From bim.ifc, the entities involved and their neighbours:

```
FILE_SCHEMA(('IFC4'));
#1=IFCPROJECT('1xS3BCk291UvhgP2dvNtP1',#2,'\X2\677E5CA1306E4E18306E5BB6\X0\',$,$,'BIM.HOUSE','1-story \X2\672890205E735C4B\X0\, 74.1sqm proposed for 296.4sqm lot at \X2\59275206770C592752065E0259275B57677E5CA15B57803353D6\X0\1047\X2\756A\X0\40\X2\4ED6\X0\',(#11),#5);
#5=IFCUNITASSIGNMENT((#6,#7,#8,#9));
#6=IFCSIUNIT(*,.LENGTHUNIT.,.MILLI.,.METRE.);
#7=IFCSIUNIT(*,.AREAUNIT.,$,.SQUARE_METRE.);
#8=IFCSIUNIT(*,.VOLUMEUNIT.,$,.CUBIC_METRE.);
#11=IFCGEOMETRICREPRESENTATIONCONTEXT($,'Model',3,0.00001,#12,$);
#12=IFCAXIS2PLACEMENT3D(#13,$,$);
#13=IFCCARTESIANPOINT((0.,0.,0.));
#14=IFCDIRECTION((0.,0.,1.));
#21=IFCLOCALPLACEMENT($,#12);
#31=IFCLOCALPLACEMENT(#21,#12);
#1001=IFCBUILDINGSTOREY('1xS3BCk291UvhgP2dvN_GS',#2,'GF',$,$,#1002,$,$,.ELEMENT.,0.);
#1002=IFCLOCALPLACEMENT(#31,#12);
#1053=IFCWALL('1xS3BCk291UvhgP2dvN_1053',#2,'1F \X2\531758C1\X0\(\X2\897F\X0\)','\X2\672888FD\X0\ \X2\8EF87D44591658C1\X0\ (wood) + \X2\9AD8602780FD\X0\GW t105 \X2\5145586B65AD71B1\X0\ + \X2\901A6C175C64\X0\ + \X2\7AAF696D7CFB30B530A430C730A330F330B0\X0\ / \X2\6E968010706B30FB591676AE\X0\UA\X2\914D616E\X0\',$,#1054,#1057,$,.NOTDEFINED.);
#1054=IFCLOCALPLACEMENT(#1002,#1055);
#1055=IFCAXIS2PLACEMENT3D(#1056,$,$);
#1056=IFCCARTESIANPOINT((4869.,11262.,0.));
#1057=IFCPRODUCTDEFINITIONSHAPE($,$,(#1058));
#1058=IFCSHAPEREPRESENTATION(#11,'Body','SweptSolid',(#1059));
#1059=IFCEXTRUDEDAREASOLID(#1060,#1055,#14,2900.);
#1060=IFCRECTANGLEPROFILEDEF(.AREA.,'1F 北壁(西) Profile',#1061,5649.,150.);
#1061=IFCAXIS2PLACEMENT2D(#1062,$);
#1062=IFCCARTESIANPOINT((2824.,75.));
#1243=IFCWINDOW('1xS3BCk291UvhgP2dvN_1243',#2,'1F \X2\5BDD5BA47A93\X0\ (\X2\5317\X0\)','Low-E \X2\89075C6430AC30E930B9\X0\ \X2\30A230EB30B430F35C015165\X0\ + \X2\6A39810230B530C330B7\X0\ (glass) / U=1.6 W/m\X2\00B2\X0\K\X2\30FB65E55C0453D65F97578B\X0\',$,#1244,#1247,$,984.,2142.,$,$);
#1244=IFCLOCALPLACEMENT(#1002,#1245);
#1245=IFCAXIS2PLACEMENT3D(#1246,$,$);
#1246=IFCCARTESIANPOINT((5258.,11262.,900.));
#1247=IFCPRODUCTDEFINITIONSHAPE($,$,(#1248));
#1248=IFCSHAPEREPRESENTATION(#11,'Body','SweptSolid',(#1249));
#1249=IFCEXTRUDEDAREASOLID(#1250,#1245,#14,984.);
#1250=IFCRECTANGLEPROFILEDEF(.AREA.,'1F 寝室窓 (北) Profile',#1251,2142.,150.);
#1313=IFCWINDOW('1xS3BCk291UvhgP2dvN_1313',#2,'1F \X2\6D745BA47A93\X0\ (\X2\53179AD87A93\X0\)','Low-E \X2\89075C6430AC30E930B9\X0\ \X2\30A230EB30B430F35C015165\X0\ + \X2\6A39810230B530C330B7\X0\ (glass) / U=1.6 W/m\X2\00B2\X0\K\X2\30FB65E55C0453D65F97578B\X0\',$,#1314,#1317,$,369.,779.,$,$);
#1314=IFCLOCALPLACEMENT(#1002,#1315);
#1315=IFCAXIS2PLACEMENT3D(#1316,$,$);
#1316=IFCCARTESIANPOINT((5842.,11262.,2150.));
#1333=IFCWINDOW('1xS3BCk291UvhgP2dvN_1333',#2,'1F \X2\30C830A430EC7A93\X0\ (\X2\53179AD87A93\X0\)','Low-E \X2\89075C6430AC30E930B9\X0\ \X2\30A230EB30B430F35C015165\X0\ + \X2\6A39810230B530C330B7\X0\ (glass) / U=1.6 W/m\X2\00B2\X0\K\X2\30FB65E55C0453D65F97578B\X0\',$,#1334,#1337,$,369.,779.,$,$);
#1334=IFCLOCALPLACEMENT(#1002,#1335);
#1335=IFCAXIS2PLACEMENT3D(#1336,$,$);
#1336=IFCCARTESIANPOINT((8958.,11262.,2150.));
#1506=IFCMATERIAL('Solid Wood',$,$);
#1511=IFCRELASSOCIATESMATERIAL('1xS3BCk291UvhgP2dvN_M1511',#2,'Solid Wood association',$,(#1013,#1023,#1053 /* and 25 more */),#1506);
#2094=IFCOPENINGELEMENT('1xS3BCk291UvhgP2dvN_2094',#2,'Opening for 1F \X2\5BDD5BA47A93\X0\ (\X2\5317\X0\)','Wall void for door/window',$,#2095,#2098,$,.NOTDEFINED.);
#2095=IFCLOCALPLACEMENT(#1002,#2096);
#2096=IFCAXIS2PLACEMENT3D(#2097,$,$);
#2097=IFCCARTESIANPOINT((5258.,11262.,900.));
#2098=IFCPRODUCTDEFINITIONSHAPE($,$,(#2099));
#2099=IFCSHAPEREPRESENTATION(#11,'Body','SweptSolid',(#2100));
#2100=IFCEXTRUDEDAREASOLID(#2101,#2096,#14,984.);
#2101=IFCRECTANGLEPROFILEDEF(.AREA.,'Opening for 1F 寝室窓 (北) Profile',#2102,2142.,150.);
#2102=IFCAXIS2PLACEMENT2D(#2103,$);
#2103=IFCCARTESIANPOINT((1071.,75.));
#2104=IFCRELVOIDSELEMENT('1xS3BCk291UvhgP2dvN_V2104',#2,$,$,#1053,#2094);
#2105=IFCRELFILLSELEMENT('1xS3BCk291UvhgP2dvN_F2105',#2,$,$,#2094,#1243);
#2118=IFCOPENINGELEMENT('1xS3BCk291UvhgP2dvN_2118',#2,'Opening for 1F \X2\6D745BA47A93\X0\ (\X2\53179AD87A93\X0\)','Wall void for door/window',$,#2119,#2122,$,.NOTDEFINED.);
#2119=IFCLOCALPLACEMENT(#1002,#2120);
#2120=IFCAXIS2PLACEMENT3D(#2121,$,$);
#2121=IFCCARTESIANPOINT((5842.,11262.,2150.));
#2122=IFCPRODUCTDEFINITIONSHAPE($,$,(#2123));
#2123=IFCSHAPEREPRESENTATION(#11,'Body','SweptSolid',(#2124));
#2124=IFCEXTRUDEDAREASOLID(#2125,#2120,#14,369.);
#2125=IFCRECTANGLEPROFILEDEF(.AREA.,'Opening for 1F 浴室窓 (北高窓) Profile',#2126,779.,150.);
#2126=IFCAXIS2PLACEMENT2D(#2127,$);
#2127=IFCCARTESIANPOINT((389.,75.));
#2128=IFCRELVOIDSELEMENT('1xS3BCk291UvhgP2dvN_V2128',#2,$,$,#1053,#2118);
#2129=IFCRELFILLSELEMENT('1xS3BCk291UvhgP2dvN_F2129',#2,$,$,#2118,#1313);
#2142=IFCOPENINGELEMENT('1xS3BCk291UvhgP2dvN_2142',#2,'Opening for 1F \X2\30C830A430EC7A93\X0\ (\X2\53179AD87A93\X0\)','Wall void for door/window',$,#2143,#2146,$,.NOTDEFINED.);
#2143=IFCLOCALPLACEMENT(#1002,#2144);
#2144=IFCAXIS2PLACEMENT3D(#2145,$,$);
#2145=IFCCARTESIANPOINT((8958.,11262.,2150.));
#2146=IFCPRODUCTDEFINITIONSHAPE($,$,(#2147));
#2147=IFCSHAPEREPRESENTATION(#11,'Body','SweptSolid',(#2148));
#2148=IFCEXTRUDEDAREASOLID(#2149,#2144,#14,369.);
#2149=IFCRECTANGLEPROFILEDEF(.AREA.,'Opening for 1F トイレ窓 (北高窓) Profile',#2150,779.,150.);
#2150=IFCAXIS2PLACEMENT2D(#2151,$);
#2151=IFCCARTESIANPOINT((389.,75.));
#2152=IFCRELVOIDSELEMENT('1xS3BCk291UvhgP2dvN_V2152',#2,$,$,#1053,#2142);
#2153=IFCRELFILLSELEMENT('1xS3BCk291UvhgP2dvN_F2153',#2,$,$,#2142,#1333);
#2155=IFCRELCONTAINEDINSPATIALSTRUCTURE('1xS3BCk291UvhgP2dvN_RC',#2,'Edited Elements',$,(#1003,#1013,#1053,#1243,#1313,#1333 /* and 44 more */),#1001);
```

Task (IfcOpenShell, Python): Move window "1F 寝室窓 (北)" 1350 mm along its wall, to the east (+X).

```python
import ifcopenshell
import ifcopenshell.api.geometry
import ifcopenshell.util.placement

model = ifcopenshell.open("bim.ifc")

window = model.by_id(1243)
opening = window.FillsVoids[0].RelatingOpeningElement
wall = opening.VoidsElements[0].RelatingBuildingElement

wall_matrix = ifcopenshell.util.placement.get_local_placement(wall.ObjectPlacement)
shift = wall_matrix[:3, 0] * 1350.0
before = ifcopenshell.util.placement.get_local_placement(window.ObjectPlacement)[:3, 3].copy()

# The window is not placed relative to its opening, so move both.
for product in (opening, window):
    matrix = ifcopenshell.util.placement.get_local_placement(product.ObjectPlacement)
    matrix[:3, 3] += shift
    ifcopenshell.api.geometry.edit_object_placement(model, product=product, matrix=matrix, is_si=False)

after = ifcopenshell.util.placement.get_local_placement(window.ObjectPlacement)[:3, 3]
print("window moved by", (after - before).round(3) + 0.0)

model.write("bim_v2.ifc")
```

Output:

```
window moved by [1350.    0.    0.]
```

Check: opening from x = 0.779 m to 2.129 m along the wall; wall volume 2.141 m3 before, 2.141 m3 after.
